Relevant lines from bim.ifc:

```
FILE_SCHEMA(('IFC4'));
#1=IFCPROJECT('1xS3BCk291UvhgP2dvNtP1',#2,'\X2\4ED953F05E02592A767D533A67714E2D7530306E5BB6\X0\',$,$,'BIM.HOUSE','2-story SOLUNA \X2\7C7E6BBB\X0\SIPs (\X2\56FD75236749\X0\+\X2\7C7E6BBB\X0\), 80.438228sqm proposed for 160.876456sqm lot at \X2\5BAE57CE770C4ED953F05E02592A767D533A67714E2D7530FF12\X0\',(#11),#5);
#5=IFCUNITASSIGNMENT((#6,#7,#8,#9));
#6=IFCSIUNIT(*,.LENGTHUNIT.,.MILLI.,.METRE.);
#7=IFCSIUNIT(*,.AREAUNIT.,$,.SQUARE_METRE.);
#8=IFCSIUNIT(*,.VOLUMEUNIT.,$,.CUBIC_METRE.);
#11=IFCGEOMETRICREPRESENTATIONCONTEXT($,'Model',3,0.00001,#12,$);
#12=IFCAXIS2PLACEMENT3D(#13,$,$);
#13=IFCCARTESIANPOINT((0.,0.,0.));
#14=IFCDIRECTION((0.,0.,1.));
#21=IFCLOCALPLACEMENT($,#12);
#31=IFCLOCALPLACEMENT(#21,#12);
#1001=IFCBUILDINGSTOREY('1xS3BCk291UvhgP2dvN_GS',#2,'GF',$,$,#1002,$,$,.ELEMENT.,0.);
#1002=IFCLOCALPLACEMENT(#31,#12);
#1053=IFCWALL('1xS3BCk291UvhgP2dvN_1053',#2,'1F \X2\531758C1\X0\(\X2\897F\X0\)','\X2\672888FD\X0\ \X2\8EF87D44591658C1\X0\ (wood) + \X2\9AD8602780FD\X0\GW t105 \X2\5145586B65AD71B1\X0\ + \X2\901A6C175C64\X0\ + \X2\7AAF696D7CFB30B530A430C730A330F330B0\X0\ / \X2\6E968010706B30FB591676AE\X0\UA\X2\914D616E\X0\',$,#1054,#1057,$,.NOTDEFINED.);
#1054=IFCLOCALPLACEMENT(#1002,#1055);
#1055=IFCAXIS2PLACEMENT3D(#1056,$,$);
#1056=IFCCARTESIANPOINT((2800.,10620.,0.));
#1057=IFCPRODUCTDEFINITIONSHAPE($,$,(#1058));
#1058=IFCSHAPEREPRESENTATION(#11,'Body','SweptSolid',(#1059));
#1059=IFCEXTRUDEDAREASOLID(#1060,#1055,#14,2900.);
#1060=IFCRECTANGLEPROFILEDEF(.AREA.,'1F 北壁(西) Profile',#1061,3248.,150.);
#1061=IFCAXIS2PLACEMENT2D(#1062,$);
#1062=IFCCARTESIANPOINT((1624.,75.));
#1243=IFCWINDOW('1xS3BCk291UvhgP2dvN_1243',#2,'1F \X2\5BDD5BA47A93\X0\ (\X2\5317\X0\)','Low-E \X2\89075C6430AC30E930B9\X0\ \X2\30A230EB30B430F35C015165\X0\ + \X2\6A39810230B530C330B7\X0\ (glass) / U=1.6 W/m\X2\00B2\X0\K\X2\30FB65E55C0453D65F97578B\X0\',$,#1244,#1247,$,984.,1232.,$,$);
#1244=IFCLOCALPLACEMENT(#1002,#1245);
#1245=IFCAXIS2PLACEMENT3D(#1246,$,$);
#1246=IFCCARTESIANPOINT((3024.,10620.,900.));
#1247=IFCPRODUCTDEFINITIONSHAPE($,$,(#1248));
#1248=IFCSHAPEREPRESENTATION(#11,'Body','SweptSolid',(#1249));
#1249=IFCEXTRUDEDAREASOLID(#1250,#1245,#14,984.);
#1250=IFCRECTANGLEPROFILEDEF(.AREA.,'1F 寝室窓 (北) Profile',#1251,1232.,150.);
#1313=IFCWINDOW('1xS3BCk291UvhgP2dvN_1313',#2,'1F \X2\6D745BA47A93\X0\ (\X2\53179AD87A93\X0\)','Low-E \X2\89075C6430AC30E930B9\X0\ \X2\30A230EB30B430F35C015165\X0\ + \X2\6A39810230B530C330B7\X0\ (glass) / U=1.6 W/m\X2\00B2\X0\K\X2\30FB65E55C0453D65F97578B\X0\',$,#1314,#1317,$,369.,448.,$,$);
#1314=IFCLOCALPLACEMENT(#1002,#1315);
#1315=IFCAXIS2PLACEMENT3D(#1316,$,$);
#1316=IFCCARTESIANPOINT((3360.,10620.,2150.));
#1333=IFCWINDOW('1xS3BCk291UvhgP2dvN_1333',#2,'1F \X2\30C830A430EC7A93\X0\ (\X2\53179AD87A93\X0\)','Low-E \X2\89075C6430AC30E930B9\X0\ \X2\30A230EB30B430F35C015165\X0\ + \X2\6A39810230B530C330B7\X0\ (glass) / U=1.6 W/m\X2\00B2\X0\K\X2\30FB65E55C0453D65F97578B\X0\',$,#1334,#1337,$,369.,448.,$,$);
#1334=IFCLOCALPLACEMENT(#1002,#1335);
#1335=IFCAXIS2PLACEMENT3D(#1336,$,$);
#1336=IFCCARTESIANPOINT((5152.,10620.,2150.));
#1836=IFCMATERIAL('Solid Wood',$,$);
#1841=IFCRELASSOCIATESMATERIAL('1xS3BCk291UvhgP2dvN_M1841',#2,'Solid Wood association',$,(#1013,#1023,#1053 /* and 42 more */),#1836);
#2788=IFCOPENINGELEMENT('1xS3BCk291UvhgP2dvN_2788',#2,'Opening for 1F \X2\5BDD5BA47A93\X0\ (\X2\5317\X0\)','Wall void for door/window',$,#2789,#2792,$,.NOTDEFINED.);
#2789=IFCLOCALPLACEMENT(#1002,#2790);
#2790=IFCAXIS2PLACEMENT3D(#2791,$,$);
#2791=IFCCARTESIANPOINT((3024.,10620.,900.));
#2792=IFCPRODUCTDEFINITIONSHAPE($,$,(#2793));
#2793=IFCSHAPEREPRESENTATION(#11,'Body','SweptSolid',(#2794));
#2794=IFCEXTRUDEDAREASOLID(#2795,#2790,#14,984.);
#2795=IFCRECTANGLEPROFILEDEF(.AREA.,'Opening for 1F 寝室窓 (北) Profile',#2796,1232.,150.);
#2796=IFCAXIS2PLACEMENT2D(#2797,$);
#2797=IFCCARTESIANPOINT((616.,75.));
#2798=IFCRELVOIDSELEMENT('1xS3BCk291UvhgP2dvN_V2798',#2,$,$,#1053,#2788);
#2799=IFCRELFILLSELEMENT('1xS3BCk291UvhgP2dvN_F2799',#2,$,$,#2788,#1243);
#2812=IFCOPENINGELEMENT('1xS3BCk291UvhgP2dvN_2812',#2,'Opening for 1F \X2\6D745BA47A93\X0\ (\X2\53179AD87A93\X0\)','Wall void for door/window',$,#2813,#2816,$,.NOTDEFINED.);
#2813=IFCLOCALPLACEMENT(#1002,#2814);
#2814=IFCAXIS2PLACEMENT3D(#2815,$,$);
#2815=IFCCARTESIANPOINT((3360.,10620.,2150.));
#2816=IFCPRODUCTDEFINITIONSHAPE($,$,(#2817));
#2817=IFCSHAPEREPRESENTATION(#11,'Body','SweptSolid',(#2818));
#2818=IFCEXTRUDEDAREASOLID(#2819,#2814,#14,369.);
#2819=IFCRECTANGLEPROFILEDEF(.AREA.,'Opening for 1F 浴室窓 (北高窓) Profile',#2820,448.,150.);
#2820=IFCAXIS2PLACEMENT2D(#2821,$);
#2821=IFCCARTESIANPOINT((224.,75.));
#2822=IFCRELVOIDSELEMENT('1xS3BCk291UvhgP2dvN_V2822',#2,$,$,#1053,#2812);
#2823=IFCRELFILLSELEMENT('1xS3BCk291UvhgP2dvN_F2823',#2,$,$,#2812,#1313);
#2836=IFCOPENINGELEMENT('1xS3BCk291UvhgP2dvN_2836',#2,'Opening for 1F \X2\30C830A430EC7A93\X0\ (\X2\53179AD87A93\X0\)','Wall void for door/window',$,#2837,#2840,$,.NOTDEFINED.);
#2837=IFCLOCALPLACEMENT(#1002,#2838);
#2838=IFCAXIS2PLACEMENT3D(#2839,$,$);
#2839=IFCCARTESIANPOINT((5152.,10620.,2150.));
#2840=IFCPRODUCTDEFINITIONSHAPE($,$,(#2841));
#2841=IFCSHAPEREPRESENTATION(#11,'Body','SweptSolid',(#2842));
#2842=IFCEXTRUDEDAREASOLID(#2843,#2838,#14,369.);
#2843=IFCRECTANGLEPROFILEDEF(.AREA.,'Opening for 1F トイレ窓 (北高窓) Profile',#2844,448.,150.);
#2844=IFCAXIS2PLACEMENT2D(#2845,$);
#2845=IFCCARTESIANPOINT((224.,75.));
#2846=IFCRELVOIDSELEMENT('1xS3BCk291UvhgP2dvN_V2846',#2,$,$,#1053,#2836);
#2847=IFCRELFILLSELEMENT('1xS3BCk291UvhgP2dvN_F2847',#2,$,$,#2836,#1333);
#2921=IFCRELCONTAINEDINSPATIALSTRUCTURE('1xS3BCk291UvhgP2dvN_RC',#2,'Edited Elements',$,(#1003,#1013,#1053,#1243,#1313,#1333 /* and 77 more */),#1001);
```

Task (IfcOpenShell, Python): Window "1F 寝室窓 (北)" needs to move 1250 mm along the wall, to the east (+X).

```python
import ifcopenshell
import ifcopenshell.api.geometry
import ifcopenshell.util.placement
import ifcopenshell.util.unit

model = ifcopenshell.open("bim.ifc")
unit_scale = ifcopenshell.util.unit.calculate_unit_scale(model)

window = model.by_guid("1xS3BCk291UvhgP2dvN_1243")
opening = window.FillsVoids[0].RelatingOpeningElement
wall = opening.VoidsElements[0].RelatingBuildingElement

wall_matrix = ifcopenshell.util.placement.get_local_placement(wall.ObjectPlacement)
shift = wall_matrix[:3, 0] * 1.25 / unit_scale
before = ifcopenshell.util.placement.get_local_placement(window.ObjectPlacement)[:3, 3].copy()

# The window is not placed relative to its opening, so move both.
for product in (opening, window):
    matrix = ifcopenshell.util.placement.get_local_placement(product.ObjectPlacement)
    matrix[:3, 3] += shift
    ifcopenshell.api.geometry.edit_object_placement(model, product=product, matrix=matrix, is_si=False)

after = ifcopenshell.util.placement.get_local_placement(window.ObjectPlacement)[:3, 3]
print("window moved by", (after - before).round(3) + 0.0)

model.write("bim_rev.ifc")
```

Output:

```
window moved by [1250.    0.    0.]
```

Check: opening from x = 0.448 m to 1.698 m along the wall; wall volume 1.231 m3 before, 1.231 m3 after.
